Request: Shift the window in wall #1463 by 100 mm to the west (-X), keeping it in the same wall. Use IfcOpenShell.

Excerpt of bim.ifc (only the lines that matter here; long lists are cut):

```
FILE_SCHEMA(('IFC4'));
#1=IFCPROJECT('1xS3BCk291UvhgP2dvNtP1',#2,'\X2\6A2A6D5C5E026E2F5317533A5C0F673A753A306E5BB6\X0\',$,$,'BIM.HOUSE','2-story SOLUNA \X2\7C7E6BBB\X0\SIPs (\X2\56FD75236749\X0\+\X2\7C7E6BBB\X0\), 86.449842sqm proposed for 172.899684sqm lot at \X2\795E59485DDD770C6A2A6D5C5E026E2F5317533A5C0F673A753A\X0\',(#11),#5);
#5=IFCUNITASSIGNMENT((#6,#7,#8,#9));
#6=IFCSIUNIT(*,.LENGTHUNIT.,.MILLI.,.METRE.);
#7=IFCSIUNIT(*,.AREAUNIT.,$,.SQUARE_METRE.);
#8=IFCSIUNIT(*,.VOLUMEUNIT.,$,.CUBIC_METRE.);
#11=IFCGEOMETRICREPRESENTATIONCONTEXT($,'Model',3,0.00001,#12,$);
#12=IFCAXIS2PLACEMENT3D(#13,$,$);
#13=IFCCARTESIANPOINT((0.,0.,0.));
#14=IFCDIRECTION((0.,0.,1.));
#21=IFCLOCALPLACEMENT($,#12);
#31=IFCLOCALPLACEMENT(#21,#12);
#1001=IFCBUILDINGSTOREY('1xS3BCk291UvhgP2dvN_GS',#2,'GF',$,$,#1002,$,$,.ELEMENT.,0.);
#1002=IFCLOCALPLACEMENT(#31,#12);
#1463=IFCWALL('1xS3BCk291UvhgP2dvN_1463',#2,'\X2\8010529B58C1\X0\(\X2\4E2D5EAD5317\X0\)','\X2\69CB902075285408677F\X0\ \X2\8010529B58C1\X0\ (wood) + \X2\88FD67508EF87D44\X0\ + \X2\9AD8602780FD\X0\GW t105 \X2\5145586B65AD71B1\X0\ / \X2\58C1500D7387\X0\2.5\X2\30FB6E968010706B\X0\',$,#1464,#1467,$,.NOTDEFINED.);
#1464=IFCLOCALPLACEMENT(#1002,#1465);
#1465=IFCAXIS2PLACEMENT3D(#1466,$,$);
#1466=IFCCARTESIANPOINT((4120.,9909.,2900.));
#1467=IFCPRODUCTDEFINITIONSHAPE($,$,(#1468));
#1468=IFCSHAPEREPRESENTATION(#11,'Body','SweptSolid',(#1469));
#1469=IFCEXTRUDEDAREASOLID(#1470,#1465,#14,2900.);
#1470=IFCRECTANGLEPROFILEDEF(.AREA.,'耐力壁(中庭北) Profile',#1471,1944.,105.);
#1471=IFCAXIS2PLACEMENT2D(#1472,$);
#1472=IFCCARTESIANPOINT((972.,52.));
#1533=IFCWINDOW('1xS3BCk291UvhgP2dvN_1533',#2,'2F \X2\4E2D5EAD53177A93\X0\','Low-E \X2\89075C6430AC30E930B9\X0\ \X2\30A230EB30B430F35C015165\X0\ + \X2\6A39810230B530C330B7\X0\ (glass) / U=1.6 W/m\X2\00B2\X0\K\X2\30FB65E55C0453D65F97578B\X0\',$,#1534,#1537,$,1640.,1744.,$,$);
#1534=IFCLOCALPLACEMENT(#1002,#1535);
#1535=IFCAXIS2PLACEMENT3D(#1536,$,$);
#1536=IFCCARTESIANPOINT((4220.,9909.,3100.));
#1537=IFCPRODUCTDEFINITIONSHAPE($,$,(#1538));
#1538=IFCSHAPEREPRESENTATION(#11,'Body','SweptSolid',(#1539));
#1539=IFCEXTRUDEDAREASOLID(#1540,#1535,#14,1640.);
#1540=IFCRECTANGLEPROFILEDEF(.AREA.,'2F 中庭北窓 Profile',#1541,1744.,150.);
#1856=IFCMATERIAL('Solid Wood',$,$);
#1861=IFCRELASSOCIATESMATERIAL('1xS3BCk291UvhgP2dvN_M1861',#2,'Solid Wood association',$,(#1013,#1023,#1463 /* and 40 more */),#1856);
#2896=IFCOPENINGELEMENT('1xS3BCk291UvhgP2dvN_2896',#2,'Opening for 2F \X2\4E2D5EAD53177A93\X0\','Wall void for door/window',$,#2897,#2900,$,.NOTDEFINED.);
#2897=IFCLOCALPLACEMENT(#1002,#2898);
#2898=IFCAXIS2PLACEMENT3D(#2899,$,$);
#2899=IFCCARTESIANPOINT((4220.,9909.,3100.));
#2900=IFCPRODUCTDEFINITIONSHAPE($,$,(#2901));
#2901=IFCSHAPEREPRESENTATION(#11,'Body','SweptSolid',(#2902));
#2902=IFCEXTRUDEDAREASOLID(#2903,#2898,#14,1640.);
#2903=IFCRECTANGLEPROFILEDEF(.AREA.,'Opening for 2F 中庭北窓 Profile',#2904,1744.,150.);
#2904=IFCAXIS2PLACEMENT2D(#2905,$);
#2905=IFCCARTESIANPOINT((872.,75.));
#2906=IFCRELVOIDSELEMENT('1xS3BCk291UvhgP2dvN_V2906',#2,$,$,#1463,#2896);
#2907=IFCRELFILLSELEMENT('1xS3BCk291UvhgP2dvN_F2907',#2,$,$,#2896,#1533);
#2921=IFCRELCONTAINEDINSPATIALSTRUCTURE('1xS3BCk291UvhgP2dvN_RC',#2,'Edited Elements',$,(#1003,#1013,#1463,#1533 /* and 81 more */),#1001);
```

```python
import ifcopenshell
import ifcopenshell.api.geometry
import ifcopenshell.util.placement
import ifcopenshell.util.unit

model = ifcopenshell.open("bim.ifc")
unit_scale = ifcopenshell.util.unit.calculate_unit_scale(model)

window = model.by_guid("1xS3BCk291UvhgP2dvN_1533")
opening = window.FillsVoids[0].RelatingOpeningElement
wall = opening.VoidsElements[0].RelatingBuildingElement

wall_matrix = ifcopenshell.util.placement.get_local_placement(wall.ObjectPlacement)
shift = wall_matrix[:3, 0] * -0.1 / unit_scale
before = ifcopenshell.util.placement.get_local_placement(window.ObjectPlacement)[:3, 3].copy()

# The window is not placed relative to its opening, so move both.
for product in (opening, window):
    matrix = ifcopenshell.util.placement.get_local_placement(product.ObjectPlacement)
    matrix[:3, 3] += shift
    ifcopenshell.api.geometry.edit_object_placement(model, product=product, matrix=matrix, is_si=False)

after = ifcopenshell.util.placement.get_local_placement(window.ObjectPlacement)[:3, 3]
print("window moved by", (after - before).round(3) + 0.0)

model.write("bim_edited.ifc")
```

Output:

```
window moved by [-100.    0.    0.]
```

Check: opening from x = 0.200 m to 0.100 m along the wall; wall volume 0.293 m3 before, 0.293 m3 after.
